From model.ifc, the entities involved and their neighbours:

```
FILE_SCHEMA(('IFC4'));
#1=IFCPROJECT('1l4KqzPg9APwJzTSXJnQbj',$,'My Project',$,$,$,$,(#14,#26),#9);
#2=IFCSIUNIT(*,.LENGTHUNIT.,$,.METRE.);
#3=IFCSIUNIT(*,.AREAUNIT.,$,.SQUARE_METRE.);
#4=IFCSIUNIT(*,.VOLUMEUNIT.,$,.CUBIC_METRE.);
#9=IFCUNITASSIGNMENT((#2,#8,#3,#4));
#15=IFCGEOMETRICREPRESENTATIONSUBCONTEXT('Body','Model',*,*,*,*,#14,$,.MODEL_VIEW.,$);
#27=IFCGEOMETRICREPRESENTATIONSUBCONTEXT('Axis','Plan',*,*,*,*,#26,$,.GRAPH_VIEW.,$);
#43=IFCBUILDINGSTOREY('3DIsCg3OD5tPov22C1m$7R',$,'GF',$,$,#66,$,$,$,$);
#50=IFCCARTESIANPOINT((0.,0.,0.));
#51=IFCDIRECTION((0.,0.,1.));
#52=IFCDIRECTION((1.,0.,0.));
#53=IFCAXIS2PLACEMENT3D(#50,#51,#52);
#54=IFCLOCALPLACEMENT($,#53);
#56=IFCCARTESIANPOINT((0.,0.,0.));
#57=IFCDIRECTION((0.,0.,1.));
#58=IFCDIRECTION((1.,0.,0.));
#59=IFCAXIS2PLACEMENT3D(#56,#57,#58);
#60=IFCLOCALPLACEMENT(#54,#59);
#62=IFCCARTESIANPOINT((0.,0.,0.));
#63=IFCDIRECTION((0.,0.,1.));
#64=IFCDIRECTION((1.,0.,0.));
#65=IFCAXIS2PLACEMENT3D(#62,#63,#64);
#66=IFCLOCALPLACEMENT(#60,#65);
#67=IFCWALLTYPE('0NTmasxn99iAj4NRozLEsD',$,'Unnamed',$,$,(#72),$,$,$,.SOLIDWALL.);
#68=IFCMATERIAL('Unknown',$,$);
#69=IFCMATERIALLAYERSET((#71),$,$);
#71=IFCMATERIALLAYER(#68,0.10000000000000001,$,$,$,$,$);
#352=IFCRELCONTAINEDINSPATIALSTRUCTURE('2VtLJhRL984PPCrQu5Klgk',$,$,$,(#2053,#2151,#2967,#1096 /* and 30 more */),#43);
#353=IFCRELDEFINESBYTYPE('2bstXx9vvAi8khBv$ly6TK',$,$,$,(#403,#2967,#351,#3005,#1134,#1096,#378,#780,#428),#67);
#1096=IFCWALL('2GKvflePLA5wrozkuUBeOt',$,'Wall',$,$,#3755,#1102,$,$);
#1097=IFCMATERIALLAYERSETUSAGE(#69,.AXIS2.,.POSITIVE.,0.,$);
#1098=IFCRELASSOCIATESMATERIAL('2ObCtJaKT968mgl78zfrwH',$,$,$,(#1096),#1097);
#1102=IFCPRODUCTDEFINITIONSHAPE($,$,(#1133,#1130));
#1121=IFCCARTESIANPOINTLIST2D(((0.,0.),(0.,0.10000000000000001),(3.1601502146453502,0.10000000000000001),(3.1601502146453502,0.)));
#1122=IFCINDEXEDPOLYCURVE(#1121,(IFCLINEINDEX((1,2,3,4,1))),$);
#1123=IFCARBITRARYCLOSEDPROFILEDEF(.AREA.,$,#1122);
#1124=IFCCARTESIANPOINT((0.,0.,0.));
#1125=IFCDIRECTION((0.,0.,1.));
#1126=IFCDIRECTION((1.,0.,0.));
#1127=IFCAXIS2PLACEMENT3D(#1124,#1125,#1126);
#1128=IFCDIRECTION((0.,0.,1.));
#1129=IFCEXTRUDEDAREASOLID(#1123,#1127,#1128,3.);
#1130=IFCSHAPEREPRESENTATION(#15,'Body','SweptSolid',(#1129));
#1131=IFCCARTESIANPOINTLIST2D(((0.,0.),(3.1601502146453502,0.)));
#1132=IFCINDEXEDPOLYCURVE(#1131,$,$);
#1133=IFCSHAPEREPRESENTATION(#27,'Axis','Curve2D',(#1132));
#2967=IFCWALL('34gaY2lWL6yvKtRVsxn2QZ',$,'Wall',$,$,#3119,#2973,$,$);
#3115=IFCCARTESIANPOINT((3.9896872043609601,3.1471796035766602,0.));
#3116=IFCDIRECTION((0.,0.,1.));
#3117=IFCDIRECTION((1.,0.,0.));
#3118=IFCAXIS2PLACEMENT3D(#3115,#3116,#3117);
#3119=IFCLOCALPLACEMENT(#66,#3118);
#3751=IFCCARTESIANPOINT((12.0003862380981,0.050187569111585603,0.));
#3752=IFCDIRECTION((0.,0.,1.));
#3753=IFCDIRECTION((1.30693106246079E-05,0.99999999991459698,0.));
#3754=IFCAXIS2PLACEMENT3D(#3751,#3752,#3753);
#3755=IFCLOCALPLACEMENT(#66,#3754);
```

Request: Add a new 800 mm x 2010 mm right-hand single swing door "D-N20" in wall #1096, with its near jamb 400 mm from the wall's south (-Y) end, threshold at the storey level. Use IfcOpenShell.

```python
import numpy as np
import ifcopenshell
import ifcopenshell.api.feature
import ifcopenshell.api.geometry
import ifcopenshell.api.root
import ifcopenshell.api.spatial
import ifcopenshell.geom
import ifcopenshell.util.element
import ifcopenshell.util.placement
import ifcopenshell.util.representation
import ifcopenshell.util.shape
import ifcopenshell.util.unit

model = ifcopenshell.open("model.ifc")
unit_scale = ifcopenshell.util.unit.calculate_unit_scale(model)
settings = ifcopenshell.geom.settings()


def volume(element):
    """Net volume in cubic metres, openings subtracted."""
    shape = ifcopenshell.geom.create_shape(settings, element)
    return ifcopenshell.util.shape.get_volume(shape.geometry)


wall = model.by_id(1096)
storey = ifcopenshell.util.element.get_container(wall, ifc_class="IfcBuildingStorey")
context = ifcopenshell.util.representation.get_context(model, "Model", "Body", "MODEL_VIEW")
before = volume(wall)

width, height, from_end, sill = 0.8, 2.01, 0.4, 0.0  # metres

# The wall runs along its own X axis, and the end named is its -X end.
wall_shape = ifcopenshell.geom.create_shape(settings, wall)
x, y, z = ifcopenshell.util.shape.get_vertices(wall_shape.geometry).T
start = x.min() + from_end
face, thickness = float(y.min()), float(y.max() - y.min())
wall_matrix = ifcopenshell.util.placement.get_local_placement(wall.ObjectPlacement)
level = ifcopenshell.util.placement.get_local_placement(storey.ObjectPlacement)[2, 3]


def in_wall(x, y):
    """Placement at x, y metres in the wall's axes, at sill height."""
    matrix = wall_matrix.copy()
    matrix[:, 3] = wall_matrix @ np.array([x / unit_scale, y / unit_scale, 0.0, 1.0])
    matrix[2, 3] = level + sill / unit_scale
    return matrix


# Opening: a box that overshoots both wall faces by 50 mm.
opening = ifcopenshell.api.root.create_entity(model, ifc_class="IfcOpeningElement", predefined_type="OPENING")
box = ifcopenshell.api.geometry.add_wall_representation(
    model, context=context, length=width, height=height, thickness=thickness + 0.1
)
ifcopenshell.api.geometry.assign_representation(model, product=opening, representation=box)
ifcopenshell.api.geometry.edit_object_placement(model, product=opening, matrix=in_wall(start, face - 0.05), is_si=False)
ifcopenshell.api.feature.add_feature(model, feature=opening, element=wall)

door = ifcopenshell.api.root.create_entity(model, ifc_class="IfcDoor", name="D-N20", predefined_type="DOOR")
door.OverallWidth, door.OverallHeight = width / unit_scale, height / unit_scale
door.OperationType = "SINGLE_SWING_RIGHT"
body = ifcopenshell.api.geometry.add_door_representation(
    model,
    context=context,
    overall_width=door.OverallWidth,
    overall_height=door.OverallHeight,
    operation_type="SINGLE_SWING_RIGHT",
    lining_properties={"LiningDepth": thickness / unit_scale, "ThresholdDepth": thickness / unit_scale},
)
ifcopenshell.api.geometry.assign_representation(model, product=door, representation=body)
ifcopenshell.api.spatial.assign_container(model, products=[door], relating_structure=storey)
ifcopenshell.api.feature.add_filling(model, opening=opening, element=door)

# The lining spans the wall, so the door starts at the wall face.
ifcopenshell.api.geometry.edit_object_placement(model, product=door, matrix=in_wall(start, face), is_si=False)

after = volume(wall)

print(f"wall volume {before:.3f} -> {after:.3f} m3")

model.write("model_edited.ifc")
```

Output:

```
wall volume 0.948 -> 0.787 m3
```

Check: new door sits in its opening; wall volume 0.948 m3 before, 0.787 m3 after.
